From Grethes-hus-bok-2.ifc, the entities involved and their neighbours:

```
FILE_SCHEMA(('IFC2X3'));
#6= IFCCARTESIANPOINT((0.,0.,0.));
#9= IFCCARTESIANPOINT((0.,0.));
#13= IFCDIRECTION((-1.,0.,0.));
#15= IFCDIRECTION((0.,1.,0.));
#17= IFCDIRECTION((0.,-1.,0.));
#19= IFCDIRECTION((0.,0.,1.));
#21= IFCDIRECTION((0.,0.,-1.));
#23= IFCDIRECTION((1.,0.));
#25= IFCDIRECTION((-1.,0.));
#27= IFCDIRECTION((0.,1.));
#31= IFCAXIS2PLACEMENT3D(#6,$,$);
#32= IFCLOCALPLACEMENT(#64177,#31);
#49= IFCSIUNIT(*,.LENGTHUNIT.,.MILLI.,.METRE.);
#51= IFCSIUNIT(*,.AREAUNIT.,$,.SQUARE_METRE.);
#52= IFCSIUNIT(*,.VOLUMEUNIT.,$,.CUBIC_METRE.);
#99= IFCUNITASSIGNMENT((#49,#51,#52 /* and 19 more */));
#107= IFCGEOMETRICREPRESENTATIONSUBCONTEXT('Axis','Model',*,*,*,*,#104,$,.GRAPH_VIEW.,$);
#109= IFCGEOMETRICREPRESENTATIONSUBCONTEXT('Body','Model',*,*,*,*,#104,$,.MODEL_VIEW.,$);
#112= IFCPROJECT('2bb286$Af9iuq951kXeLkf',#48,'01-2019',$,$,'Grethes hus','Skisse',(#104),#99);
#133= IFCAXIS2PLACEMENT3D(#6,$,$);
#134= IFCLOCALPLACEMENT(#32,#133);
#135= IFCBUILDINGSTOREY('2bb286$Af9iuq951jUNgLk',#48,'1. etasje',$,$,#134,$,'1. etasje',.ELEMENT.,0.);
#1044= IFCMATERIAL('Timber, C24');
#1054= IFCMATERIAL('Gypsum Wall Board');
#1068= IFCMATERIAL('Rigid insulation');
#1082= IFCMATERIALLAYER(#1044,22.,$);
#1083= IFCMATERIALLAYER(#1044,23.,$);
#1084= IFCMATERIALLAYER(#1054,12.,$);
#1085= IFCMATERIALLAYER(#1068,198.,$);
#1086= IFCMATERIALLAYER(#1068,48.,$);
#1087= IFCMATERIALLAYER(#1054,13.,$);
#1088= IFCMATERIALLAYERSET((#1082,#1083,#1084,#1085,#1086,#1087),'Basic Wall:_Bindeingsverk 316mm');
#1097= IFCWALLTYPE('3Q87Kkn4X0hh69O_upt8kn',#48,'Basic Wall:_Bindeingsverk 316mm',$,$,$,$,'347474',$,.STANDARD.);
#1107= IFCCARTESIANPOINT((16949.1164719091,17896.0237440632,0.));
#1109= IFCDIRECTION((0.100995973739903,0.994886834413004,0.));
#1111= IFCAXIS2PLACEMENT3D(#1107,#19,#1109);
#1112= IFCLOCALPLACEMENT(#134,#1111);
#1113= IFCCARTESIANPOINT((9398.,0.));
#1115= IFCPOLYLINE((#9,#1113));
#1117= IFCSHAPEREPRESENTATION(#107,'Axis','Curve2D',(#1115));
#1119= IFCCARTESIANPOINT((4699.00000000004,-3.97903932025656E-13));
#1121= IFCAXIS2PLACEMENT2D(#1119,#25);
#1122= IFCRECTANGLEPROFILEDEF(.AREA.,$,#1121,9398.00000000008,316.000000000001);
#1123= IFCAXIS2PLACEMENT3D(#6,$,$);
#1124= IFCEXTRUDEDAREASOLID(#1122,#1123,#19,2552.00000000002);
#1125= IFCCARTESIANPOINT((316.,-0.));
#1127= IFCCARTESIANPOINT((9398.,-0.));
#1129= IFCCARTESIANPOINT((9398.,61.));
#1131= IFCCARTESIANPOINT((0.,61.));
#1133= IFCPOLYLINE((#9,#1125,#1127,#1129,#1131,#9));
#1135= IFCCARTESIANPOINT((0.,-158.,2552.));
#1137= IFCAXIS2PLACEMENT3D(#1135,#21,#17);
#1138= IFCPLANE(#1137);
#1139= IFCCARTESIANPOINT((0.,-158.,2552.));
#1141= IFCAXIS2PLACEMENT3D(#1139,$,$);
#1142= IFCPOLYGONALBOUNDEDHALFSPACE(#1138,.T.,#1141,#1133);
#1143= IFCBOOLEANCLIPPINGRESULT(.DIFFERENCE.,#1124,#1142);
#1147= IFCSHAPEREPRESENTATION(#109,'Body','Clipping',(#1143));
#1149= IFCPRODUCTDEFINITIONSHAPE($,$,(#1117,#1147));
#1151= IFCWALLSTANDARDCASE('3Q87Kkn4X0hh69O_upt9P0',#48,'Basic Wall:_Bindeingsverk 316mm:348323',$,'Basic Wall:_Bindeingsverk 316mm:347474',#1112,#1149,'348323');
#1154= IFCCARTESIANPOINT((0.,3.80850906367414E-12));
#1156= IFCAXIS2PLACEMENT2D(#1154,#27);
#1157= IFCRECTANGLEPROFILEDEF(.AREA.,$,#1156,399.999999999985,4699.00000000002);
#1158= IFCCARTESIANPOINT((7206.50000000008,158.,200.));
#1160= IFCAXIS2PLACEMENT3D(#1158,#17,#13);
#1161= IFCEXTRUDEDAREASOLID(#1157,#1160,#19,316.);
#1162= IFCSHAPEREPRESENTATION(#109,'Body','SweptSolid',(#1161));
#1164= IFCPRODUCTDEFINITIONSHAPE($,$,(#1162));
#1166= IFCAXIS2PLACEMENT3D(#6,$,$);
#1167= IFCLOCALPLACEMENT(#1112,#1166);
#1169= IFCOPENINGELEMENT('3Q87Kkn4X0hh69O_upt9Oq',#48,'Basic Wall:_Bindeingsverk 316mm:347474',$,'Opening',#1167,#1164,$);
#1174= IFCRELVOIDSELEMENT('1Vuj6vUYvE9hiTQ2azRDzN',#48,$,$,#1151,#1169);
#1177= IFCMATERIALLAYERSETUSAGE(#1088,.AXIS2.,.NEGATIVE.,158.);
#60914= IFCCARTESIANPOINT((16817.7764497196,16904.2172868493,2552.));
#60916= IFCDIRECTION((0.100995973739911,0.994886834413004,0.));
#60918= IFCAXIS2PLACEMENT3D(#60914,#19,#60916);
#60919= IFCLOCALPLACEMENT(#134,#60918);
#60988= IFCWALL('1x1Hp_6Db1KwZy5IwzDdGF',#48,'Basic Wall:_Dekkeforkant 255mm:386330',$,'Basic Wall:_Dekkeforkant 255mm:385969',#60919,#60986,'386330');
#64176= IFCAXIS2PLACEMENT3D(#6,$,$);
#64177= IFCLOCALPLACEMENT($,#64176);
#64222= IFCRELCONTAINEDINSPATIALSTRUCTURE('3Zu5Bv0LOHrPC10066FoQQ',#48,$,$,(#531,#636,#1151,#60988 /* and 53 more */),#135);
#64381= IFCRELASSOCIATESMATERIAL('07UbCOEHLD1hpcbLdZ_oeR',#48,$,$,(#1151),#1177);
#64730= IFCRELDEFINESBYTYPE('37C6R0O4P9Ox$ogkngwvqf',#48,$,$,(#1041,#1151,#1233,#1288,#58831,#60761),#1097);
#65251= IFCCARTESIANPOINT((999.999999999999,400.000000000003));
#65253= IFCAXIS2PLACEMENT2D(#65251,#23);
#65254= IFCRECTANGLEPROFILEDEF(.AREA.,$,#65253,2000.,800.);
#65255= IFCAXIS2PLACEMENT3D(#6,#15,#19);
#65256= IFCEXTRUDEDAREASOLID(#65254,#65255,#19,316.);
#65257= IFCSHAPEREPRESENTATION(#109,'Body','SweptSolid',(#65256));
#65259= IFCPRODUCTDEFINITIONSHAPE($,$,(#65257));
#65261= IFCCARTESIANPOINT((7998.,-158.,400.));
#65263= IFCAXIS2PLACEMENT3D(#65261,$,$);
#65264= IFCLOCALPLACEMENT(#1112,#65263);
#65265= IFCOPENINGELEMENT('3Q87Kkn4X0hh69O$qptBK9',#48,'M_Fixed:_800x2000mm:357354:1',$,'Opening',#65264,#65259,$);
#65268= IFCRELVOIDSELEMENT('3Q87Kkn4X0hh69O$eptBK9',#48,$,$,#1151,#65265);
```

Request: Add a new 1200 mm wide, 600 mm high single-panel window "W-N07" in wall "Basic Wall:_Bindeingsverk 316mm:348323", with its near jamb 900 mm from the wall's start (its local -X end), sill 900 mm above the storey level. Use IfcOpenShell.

```python
import numpy as np
import ifcopenshell
import ifcopenshell.api.feature
import ifcopenshell.api.geometry
import ifcopenshell.api.root
import ifcopenshell.api.spatial
import ifcopenshell.api.type
import ifcopenshell.geom
import ifcopenshell.util.element
import ifcopenshell.util.placement
import ifcopenshell.util.representation
import ifcopenshell.util.shape
import ifcopenshell.util.unit

model = ifcopenshell.open("Grethes-hus-bok-2.ifc")
unit_scale = ifcopenshell.util.unit.calculate_unit_scale(model)
settings = ifcopenshell.geom.settings()


def volume(element):
    """Net volume in cubic metres, openings subtracted."""
    shape = ifcopenshell.geom.create_shape(settings, element)
    return ifcopenshell.util.shape.get_volume(shape.geometry)


wall = model.by_guid("3Q87Kkn4X0hh69O_upt9P0")
storey = ifcopenshell.util.element.get_container(wall, ifc_class="IfcBuildingStorey")
context = ifcopenshell.util.representation.get_context(model, "Model", "Body", "MODEL_VIEW")
before = volume(wall)

width, height, from_end, sill = 1.2, 0.6, 0.9, 0.9  # metres

# The wall runs along its own X axis, and the end named is its -X end.
wall_shape = ifcopenshell.geom.create_shape(settings, wall)
x, y, z = ifcopenshell.util.shape.get_vertices(wall_shape.geometry).T
start = x.min() + from_end
face, thickness = float(y.min()), float(y.max() - y.min())
wall_matrix = ifcopenshell.util.placement.get_local_placement(wall.ObjectPlacement)
level = ifcopenshell.util.placement.get_local_placement(storey.ObjectPlacement)[2, 3]


def in_wall(x, y):
    """Placement at x, y metres in the wall's axes, at sill height."""
    matrix = wall_matrix.copy()
    matrix[:, 3] = wall_matrix @ np.array([x / unit_scale, y / unit_scale, 0.0, 1.0])
    matrix[2, 3] = level + sill / unit_scale
    return matrix


# Opening: a box that overshoots both wall faces by 50 mm.
opening = ifcopenshell.api.root.create_entity(model, ifc_class="IfcOpeningElement")
box = ifcopenshell.api.geometry.add_wall_representation(
    model, context=context, length=width, height=height, thickness=thickness + 0.1
)
ifcopenshell.api.geometry.assign_representation(model, product=opening, representation=box)
ifcopenshell.api.geometry.edit_object_placement(model, product=opening, matrix=in_wall(start, face - 0.05), is_si=False)
ifcopenshell.api.feature.add_feature(model, feature=opening, element=wall)

window = ifcopenshell.api.root.create_entity(model, ifc_class="IfcWindow", name="W-N07")
window.OverallWidth, window.OverallHeight = width / unit_scale, height / unit_scale
body = ifcopenshell.api.geometry.add_window_representation(
    model,
    context=context,
    overall_width=window.OverallWidth,
    overall_height=window.OverallHeight,
    partition_type="SINGLE_PANEL",
)
ifcopenshell.api.geometry.assign_representation(model, product=window, representation=body)
ifcopenshell.api.spatial.assign_container(model, products=[window], relating_structure=storey)
fills = ifcopenshell.api.feature.add_filling(model, opening=opening, element=window)
fills.OwnerHistory = window.OwnerHistory  # required in IFC2X3

# IFC2X3 keeps the operation on the window style.
style = ifcopenshell.api.root.create_entity(model, ifc_class="IfcWindowStyle", name="W-N07")
style.OperationType, style.ConstructionType = "SINGLE_PANEL", "NOTDEFINED"
style.ParameterTakesPrecedence = style.Sizeable = False
ifcopenshell.api.type.assign_type(model, related_objects=[window], relating_type=style)

# Centre the window in the wall's thickness.
ifcopenshell.api.geometry.edit_object_placement(model, product=window, matrix=in_wall(start, face), is_si=False)
window_shape = ifcopenshell.geom.create_shape(settings, window)
depth = ifcopenshell.util.shape.get_vertices(window_shape.geometry)[:, 1]
offset = face + thickness / 2 - (depth.min() + depth.max()) / 2
ifcopenshell.api.geometry.edit_object_placement(model, product=window, matrix=in_wall(start, offset), is_si=False)

after = volume(wall)

print(f"wall volume {before:.3f} -> {after:.3f} m3")

model.write("Grethes-hus-bok-2_v2.ifc")
```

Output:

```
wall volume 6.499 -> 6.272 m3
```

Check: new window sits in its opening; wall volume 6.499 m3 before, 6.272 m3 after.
